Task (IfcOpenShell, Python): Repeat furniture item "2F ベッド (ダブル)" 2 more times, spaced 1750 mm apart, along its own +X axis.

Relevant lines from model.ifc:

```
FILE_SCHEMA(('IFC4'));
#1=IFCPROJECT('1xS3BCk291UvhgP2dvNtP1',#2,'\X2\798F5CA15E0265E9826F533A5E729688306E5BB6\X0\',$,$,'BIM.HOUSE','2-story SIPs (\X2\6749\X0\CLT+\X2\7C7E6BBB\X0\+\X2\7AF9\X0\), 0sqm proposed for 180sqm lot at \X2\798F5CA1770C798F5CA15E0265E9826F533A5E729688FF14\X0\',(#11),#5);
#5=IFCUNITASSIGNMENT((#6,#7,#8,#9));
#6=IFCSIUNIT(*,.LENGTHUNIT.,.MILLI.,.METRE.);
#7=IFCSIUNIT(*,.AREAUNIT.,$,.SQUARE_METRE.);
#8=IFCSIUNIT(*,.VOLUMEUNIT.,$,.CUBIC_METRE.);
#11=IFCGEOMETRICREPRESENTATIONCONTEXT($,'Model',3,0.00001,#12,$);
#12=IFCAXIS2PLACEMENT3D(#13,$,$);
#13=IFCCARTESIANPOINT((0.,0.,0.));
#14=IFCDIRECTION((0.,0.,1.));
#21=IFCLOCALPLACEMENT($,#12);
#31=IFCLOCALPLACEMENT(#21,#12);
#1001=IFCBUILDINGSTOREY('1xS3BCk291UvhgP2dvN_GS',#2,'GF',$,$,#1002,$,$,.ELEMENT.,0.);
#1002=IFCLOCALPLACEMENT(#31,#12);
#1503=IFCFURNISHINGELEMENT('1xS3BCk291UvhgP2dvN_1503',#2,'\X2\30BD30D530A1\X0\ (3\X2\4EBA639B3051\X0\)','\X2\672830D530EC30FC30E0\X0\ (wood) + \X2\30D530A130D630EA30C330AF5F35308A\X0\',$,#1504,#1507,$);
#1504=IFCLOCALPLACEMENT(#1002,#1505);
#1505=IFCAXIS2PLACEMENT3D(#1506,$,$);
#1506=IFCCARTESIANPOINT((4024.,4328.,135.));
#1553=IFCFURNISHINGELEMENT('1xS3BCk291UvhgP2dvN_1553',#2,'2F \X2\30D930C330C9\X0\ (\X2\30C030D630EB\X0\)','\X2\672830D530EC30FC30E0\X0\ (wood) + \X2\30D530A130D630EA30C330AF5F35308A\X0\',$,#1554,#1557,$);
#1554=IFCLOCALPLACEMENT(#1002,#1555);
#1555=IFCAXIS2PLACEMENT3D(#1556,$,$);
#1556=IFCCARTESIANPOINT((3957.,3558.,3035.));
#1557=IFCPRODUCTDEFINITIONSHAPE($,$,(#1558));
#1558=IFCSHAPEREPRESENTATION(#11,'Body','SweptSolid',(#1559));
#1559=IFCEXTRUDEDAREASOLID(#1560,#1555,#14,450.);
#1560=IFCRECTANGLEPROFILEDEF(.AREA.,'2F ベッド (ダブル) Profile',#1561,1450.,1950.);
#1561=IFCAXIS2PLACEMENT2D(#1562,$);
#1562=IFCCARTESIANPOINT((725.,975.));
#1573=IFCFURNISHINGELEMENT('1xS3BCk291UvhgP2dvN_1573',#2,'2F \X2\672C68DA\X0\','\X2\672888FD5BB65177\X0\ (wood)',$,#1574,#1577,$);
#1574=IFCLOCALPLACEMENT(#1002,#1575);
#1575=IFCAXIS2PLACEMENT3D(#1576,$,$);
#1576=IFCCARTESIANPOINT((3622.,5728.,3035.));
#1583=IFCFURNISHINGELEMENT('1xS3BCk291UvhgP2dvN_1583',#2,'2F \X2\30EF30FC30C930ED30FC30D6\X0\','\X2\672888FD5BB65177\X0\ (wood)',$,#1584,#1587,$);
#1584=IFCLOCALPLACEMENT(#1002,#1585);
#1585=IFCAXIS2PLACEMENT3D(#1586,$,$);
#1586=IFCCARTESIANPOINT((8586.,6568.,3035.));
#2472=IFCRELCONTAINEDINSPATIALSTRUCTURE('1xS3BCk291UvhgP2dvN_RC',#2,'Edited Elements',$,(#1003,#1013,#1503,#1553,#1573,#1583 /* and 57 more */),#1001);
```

```python
import ifcopenshell
import ifcopenshell.api.geometry
import ifcopenshell.api.root
import ifcopenshell.util.element
import ifcopenshell.util.placement

model = ifcopenshell.open("model.ifc")


def reuse_history(source, copy):
    """copy_class also copies each property set's owner history, people and application; keep the originals."""
    for rel in copy.IsDefinedBy:
        if rel.is_a("IfcRelDefinesByProperties") and (history := rel.RelatingPropertyDefinition.OwnerHistory):
            rel.RelatingPropertyDefinition.OwnerHistory = source.OwnerHistory
            ifcopenshell.util.element.remove_deep2(model, history)


source = model.by_guid("1xS3BCk291UvhgP2dvN_1553")
base = ifcopenshell.util.placement.get_local_placement(source.ObjectPlacement)
step = base[:3, 0] * 1750.0

for i in range(1, 3):
    copy = ifcopenshell.api.root.copy_class(model, product=source)
    copy.Representation = ifcopenshell.util.element.copy_deep(
        model, source.Representation, exclude=["IfcGeometricRepresentationContext", "IfcRepresentationMap"]
    )
    reuse_history(source, copy)
    matrix = base.copy()
    matrix[:3, 3] += i * step
    print("added at", matrix[:3, 3].round(3) + 0.0)
    ifcopenshell.api.geometry.edit_object_placement(model, product=copy, matrix=matrix, is_si=False)

model.write("model_v2.ifc")
```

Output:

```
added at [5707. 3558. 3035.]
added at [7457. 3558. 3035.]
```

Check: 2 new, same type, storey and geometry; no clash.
